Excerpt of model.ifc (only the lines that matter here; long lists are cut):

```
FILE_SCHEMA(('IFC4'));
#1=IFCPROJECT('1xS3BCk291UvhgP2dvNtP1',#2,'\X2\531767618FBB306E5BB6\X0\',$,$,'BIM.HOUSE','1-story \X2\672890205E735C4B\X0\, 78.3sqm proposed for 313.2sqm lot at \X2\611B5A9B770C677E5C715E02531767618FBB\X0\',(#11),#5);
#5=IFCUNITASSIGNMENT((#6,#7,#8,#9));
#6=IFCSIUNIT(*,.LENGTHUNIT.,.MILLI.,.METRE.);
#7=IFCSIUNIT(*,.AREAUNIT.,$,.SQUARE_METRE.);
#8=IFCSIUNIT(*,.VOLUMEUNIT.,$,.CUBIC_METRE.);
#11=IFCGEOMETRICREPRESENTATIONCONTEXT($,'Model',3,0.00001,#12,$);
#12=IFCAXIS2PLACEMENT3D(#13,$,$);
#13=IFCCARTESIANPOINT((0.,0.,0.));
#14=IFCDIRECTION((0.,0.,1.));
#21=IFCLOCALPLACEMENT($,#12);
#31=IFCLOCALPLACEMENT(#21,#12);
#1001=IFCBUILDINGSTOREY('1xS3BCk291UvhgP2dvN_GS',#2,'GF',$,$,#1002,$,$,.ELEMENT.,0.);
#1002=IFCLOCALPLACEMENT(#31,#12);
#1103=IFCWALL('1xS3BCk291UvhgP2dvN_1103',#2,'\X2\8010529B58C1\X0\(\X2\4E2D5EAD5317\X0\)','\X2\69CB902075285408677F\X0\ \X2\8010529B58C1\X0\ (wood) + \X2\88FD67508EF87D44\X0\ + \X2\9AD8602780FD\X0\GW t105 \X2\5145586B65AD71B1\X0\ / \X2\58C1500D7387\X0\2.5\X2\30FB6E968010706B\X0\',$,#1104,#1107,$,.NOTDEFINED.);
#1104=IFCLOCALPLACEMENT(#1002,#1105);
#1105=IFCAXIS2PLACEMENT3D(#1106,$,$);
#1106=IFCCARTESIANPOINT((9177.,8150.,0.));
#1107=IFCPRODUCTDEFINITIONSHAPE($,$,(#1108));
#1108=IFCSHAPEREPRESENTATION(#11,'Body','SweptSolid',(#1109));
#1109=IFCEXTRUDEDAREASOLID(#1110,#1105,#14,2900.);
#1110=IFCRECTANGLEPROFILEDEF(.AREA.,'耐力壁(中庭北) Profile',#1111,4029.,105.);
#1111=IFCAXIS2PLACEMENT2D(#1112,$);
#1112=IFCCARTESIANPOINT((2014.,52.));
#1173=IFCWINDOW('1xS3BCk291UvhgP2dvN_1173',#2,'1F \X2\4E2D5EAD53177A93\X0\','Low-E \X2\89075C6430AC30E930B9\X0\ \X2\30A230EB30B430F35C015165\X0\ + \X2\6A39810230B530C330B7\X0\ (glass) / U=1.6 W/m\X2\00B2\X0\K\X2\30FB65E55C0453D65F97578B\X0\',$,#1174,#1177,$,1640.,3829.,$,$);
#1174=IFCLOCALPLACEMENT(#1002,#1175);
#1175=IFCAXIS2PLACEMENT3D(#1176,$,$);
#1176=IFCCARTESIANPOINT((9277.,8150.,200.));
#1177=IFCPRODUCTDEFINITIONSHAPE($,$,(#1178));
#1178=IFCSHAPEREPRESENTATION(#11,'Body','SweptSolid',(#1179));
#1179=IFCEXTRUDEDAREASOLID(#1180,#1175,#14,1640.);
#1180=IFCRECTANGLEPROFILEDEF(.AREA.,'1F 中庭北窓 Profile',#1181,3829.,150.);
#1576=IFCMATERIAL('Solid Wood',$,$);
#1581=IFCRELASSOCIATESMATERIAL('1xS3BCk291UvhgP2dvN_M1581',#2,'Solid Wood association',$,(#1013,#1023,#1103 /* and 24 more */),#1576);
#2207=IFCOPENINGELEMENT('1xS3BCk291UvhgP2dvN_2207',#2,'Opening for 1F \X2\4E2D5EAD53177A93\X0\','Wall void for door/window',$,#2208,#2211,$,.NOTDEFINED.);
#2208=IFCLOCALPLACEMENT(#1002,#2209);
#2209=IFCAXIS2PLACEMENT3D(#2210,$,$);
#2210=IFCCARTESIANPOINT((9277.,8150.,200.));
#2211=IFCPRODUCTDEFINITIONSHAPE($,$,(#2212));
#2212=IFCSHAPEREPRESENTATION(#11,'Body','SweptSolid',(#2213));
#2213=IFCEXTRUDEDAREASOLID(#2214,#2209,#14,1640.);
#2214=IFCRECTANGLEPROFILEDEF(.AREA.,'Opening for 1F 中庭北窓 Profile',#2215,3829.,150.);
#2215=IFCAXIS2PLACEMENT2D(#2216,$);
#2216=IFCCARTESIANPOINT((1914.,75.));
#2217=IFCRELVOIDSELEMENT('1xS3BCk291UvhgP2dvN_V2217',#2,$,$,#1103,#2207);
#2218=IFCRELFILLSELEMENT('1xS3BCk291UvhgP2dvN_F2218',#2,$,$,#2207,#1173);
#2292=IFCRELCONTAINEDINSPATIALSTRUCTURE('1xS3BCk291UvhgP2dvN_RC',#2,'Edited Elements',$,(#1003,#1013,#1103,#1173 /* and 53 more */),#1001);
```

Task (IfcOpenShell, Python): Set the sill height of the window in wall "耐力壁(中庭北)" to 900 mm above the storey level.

```python
import numpy as np
import ifcopenshell
import ifcopenshell.api.geometry
import ifcopenshell.geom
import ifcopenshell.util.element
import ifcopenshell.util.placement
import ifcopenshell.util.shape
import ifcopenshell.util.unit

model = ifcopenshell.open("model.ifc")
unit_scale = ifcopenshell.util.unit.calculate_unit_scale(model)

window = model.by_guid("1xS3BCk291UvhgP2dvN_1173")
opening = window.FillsVoids[0].RelatingOpeningElement
storey = ifcopenshell.util.element.get_container(window, ifc_class="IfcBuildingStorey")
level = ifcopenshell.util.placement.get_local_placement(storey.ObjectPlacement)[2, 3]

# The opening's origin need not be at the sill, so measure its lowest point.
shape = ifcopenshell.geom.create_shape(ifcopenshell.geom.settings(), opening)
bottom = ifcopenshell.util.shape.get_shape_bottom_elevation(shape, shape.geometry) / unit_scale
dz = level + 900.0 - bottom

shift = np.array([0.0, 0.0, dz])
# The window is not placed relative to its opening, so move both.
for product in (opening, window):
    matrix = ifcopenshell.util.placement.get_local_placement(product.ObjectPlacement)
    matrix[:3, 3] += shift
    ifcopenshell.api.geometry.edit_object_placement(model, product=product, matrix=matrix, is_si=False)

print(f"moved by {dz * unit_scale:+.3f} m")

model.write("model_updated.ifc")
```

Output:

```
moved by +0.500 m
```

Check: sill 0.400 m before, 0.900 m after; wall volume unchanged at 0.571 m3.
